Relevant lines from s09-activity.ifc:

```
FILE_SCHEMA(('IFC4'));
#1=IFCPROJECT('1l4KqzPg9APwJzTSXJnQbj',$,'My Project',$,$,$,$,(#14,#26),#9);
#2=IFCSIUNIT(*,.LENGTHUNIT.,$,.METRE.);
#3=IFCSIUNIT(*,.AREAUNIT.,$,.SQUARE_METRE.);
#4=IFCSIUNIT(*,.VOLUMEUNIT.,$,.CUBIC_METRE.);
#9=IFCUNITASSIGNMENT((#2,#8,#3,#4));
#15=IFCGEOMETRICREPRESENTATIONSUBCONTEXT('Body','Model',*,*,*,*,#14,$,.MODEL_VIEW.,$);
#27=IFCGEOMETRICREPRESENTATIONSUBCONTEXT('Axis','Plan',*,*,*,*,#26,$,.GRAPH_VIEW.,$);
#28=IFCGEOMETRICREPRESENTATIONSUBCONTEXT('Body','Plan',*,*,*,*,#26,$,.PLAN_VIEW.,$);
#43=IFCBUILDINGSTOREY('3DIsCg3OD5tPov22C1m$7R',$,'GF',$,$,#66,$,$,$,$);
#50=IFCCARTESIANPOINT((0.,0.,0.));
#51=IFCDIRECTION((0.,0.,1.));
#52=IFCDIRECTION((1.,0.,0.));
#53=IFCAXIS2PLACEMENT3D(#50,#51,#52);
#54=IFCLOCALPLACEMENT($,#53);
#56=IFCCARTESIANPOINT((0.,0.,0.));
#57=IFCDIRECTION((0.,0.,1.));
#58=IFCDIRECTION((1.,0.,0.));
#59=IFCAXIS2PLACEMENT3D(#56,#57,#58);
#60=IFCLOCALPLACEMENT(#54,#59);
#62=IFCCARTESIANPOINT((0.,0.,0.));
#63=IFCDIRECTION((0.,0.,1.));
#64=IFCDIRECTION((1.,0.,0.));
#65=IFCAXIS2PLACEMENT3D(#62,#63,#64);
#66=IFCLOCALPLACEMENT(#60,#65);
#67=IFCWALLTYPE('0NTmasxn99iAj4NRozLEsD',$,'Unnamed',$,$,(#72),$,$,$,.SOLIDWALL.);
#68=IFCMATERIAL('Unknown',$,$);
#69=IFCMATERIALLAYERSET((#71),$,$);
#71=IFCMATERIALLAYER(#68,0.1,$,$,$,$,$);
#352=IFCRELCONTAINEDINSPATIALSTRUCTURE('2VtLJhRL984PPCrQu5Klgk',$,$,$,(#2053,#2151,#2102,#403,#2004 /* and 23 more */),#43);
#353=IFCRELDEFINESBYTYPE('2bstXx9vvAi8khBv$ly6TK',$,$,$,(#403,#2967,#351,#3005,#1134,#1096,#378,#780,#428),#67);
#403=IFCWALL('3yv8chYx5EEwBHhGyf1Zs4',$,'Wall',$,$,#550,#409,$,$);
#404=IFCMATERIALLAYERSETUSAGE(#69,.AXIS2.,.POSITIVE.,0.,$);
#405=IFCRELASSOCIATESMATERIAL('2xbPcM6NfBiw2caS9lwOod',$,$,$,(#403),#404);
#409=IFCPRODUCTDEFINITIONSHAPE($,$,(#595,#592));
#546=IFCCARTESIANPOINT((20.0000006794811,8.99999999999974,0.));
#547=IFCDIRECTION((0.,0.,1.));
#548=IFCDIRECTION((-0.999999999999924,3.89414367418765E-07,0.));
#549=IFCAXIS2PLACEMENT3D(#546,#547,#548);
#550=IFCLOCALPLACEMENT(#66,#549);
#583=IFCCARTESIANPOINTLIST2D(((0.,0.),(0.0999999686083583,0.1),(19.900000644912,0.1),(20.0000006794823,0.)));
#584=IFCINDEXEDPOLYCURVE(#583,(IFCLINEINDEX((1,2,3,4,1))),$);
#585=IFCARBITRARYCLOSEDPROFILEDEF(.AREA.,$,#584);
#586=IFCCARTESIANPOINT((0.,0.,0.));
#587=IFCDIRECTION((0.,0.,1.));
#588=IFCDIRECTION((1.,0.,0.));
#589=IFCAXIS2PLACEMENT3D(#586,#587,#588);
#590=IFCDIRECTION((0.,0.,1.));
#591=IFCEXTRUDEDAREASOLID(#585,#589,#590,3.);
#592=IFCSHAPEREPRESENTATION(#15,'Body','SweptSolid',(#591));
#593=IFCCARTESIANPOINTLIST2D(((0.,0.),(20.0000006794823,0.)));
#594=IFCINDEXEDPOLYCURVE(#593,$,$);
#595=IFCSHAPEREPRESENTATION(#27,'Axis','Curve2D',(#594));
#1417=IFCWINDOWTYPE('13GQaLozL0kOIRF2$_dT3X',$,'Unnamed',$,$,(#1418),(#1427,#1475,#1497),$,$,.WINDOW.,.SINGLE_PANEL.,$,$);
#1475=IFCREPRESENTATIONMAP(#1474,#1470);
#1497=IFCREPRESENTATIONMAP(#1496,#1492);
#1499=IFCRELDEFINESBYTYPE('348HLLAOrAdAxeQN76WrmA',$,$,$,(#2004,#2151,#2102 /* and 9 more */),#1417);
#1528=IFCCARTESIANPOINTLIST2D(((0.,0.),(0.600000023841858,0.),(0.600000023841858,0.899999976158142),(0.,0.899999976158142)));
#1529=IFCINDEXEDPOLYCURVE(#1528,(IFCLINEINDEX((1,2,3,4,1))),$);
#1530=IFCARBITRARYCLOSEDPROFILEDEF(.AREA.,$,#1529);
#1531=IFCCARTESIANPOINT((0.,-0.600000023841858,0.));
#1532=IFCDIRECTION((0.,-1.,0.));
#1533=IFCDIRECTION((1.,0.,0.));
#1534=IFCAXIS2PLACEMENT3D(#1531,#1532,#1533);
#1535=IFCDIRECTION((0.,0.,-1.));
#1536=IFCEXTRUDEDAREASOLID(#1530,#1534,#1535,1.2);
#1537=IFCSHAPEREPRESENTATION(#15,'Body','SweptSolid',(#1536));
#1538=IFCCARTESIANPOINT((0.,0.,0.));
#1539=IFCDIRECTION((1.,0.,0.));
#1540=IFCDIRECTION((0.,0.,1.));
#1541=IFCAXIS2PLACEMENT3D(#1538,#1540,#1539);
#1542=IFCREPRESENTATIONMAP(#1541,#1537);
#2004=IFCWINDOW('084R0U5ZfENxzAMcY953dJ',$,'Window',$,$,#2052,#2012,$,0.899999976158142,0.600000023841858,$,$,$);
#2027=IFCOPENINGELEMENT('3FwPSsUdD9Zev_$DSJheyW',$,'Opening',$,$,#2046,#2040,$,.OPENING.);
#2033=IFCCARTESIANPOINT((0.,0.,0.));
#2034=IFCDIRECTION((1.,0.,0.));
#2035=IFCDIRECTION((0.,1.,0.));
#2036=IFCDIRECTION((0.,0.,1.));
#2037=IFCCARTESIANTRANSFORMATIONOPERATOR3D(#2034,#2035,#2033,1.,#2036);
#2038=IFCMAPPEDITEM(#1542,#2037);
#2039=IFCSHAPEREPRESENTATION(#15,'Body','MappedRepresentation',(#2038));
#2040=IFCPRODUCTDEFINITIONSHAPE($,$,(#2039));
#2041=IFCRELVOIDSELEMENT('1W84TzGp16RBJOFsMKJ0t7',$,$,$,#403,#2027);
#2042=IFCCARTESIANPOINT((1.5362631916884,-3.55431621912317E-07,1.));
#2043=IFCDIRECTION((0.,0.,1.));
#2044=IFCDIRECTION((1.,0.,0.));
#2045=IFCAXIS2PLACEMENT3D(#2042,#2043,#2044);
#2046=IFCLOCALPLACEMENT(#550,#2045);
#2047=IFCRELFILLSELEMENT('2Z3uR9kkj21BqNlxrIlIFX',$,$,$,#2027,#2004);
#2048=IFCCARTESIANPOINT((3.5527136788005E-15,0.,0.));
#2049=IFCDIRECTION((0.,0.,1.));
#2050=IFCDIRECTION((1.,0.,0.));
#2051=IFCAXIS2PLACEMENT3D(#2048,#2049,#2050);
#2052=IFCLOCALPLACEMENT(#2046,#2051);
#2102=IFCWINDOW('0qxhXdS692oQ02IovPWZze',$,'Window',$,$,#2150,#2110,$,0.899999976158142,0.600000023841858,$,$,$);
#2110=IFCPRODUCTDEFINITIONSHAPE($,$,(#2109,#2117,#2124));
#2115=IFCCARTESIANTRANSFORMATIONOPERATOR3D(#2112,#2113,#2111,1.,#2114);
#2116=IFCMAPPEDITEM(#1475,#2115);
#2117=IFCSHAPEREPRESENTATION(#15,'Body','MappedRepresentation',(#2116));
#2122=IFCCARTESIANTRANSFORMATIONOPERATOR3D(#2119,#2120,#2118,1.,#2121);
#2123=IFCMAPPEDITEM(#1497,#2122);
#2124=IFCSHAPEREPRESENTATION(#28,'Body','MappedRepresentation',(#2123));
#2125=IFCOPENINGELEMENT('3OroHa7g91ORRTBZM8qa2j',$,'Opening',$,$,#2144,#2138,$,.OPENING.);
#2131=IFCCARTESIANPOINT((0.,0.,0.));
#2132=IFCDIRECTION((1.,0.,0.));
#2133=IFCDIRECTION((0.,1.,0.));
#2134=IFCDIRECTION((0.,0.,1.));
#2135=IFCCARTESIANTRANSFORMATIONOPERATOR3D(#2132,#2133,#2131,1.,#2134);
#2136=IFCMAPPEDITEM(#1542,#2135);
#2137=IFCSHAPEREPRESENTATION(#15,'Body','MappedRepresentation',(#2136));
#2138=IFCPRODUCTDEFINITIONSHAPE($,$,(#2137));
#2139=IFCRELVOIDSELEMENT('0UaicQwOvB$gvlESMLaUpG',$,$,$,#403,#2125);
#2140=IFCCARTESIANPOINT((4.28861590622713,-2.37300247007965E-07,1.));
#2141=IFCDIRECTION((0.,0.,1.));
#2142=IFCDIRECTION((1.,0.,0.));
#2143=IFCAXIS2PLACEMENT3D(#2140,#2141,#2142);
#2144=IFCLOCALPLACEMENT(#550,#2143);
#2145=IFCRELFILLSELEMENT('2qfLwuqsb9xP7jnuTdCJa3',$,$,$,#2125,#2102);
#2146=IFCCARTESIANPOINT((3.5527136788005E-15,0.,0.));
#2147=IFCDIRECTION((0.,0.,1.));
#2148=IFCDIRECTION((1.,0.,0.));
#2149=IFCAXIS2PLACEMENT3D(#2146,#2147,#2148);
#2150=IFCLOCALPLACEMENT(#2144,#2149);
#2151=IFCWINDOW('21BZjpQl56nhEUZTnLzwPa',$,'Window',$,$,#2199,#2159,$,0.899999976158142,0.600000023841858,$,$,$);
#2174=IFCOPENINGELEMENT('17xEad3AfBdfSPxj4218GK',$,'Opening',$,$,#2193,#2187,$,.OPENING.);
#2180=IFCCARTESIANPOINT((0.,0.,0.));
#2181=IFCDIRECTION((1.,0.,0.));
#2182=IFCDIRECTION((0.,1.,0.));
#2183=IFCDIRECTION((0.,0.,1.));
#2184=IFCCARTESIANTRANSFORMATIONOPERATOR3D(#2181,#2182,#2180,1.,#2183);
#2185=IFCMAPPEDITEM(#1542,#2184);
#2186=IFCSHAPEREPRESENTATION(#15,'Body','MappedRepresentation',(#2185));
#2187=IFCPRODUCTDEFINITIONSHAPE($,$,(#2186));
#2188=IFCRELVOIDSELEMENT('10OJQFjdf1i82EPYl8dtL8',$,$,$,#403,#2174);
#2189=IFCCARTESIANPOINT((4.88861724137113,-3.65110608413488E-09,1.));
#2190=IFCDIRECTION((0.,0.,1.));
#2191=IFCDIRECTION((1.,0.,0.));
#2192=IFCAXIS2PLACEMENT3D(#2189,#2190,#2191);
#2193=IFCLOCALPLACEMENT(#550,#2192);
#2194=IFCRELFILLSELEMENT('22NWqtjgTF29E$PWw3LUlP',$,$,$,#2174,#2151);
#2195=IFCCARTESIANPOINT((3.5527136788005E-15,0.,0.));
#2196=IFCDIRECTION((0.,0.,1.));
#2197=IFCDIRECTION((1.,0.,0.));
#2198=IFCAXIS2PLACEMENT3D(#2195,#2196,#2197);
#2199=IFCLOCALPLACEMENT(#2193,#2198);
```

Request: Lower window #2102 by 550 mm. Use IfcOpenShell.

```python
import numpy as np
import ifcopenshell
import ifcopenshell.api.geometry
import ifcopenshell.util.placement
import ifcopenshell.util.unit

model = ifcopenshell.open("s09-activity.ifc")
unit_scale = ifcopenshell.util.unit.calculate_unit_scale(model)

window = model.by_id(2102)
opening = window.FillsVoids[0].RelatingOpeningElement
dz = -0.55 / unit_scale

shift = np.array([0.0, 0.0, dz])
# The window is placed relative to its opening, so it follows when the opening moves.
matrix = ifcopenshell.util.placement.get_local_placement(opening.ObjectPlacement)
matrix[:3, 3] += shift
ifcopenshell.api.geometry.edit_object_placement(
    model, product=opening, matrix=matrix, is_si=False, should_transform_children=True
)

print(f"moved by {dz * unit_scale:+.3f} m")

model.write("s09-activity_edited.ifc")
```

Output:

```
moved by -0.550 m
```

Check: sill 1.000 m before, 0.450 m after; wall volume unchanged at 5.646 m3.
